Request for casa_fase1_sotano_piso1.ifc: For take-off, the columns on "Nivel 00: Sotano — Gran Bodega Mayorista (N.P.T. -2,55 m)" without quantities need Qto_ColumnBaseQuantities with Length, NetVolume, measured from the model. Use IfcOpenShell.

First a look at what the model holds.

```python
import ifcopenshell
import ifcopenshell.util.element
import ifcopenshell.util.unit

model = ifcopenshell.open("casa_fase1_sotano_piso1.ifc")
print(model.schema)
for unit_type in ("LENGTHUNIT", "AREAUNIT", "VOLUMEUNIT"):
    print(unit_type, ifcopenshell.util.unit.calculate_unit_scale(model, unit_type))
storey = next(s for s in model.by_type("IfcBuildingStorey") if s.Name == "Nivel 00: Sotano — Gran Bodega Mayorista (N.P.T. -2,55 m)")
columns = [e for e in ifcopenshell.util.element.get_decomposition(storey) if e.is_a("IfcColumn")]
for e in sorted(columns, key=lambda e: e.id()):
    print(e.id(), e.is_a(), e.Name, list(ifcopenshell.util.element.get_psets(e, qtos_only=True)), sep=" | ")
```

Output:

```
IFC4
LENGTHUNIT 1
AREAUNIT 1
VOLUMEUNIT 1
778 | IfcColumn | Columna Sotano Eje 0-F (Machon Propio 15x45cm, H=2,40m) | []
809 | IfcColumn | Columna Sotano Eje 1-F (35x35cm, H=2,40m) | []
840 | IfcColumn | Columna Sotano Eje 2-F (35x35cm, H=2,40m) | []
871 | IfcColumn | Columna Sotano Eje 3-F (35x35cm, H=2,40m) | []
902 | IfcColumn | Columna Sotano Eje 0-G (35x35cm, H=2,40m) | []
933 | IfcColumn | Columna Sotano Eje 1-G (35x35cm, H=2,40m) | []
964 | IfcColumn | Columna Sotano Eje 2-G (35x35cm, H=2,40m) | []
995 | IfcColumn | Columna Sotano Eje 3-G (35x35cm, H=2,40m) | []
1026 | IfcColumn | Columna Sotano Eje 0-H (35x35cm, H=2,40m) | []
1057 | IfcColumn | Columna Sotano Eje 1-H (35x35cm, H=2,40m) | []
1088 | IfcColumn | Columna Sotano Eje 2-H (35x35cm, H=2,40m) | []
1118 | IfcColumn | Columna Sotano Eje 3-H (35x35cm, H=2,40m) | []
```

```python
import ifcopenshell
import ifcopenshell.api.pset
import ifcopenshell.geom
import ifcopenshell.util.element
import ifcopenshell.util.shape
import ifcopenshell.util.unit

model = ifcopenshell.open("casa_fase1_sotano_piso1.ifc")
unit_scale = ifcopenshell.util.unit.calculate_unit_scale(model)
volume_scale = ifcopenshell.util.unit.calculate_unit_scale(model, "VOLUMEUNIT")
settings = ifcopenshell.geom.settings()

storey = next(s for s in model.by_type("IfcBuildingStorey") if s.Name == "Nivel 00: Sotano — Gran Bodega Mayorista (N.P.T. -2,55 m)")
columns = [e for e in ifcopenshell.util.element.get_decomposition(storey) if e.is_a("IfcColumn")]

for e in sorted(columns, key=lambda e: e.id()):
    if ifcopenshell.util.element.get_psets(e, qtos_only=True, should_inherit=False):
        continue
    # Geometry comes back in metres, in the element's own axes.
    shape = ifcopenshell.geom.create_shape(settings, e)
    values = {
        "Length": ifcopenshell.util.shape.get_z(shape.geometry) / unit_scale,
        "NetVolume": ifcopenshell.util.shape.get_volume(shape.geometry) / volume_scale,
    }
    qto = ifcopenshell.api.pset.add_qto(model, product=e, name="Qto_ColumnBaseQuantities")
    ifcopenshell.api.pset.edit_qto(model, qto=qto, properties=values)
    print(e.id(), {k: round(v, 3) for k, v in values.items()})

model.write("casa_fase1_sotano_piso1_updated.ifc")
```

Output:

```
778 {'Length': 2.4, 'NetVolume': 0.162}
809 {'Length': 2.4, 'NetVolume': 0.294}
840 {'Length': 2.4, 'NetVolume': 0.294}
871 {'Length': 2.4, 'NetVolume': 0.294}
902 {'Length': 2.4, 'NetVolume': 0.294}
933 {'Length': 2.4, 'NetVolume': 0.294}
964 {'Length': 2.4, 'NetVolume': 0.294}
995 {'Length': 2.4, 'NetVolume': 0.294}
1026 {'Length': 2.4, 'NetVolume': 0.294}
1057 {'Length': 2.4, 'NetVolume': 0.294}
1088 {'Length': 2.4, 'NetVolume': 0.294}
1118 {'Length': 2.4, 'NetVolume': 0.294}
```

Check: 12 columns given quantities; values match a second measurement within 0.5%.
